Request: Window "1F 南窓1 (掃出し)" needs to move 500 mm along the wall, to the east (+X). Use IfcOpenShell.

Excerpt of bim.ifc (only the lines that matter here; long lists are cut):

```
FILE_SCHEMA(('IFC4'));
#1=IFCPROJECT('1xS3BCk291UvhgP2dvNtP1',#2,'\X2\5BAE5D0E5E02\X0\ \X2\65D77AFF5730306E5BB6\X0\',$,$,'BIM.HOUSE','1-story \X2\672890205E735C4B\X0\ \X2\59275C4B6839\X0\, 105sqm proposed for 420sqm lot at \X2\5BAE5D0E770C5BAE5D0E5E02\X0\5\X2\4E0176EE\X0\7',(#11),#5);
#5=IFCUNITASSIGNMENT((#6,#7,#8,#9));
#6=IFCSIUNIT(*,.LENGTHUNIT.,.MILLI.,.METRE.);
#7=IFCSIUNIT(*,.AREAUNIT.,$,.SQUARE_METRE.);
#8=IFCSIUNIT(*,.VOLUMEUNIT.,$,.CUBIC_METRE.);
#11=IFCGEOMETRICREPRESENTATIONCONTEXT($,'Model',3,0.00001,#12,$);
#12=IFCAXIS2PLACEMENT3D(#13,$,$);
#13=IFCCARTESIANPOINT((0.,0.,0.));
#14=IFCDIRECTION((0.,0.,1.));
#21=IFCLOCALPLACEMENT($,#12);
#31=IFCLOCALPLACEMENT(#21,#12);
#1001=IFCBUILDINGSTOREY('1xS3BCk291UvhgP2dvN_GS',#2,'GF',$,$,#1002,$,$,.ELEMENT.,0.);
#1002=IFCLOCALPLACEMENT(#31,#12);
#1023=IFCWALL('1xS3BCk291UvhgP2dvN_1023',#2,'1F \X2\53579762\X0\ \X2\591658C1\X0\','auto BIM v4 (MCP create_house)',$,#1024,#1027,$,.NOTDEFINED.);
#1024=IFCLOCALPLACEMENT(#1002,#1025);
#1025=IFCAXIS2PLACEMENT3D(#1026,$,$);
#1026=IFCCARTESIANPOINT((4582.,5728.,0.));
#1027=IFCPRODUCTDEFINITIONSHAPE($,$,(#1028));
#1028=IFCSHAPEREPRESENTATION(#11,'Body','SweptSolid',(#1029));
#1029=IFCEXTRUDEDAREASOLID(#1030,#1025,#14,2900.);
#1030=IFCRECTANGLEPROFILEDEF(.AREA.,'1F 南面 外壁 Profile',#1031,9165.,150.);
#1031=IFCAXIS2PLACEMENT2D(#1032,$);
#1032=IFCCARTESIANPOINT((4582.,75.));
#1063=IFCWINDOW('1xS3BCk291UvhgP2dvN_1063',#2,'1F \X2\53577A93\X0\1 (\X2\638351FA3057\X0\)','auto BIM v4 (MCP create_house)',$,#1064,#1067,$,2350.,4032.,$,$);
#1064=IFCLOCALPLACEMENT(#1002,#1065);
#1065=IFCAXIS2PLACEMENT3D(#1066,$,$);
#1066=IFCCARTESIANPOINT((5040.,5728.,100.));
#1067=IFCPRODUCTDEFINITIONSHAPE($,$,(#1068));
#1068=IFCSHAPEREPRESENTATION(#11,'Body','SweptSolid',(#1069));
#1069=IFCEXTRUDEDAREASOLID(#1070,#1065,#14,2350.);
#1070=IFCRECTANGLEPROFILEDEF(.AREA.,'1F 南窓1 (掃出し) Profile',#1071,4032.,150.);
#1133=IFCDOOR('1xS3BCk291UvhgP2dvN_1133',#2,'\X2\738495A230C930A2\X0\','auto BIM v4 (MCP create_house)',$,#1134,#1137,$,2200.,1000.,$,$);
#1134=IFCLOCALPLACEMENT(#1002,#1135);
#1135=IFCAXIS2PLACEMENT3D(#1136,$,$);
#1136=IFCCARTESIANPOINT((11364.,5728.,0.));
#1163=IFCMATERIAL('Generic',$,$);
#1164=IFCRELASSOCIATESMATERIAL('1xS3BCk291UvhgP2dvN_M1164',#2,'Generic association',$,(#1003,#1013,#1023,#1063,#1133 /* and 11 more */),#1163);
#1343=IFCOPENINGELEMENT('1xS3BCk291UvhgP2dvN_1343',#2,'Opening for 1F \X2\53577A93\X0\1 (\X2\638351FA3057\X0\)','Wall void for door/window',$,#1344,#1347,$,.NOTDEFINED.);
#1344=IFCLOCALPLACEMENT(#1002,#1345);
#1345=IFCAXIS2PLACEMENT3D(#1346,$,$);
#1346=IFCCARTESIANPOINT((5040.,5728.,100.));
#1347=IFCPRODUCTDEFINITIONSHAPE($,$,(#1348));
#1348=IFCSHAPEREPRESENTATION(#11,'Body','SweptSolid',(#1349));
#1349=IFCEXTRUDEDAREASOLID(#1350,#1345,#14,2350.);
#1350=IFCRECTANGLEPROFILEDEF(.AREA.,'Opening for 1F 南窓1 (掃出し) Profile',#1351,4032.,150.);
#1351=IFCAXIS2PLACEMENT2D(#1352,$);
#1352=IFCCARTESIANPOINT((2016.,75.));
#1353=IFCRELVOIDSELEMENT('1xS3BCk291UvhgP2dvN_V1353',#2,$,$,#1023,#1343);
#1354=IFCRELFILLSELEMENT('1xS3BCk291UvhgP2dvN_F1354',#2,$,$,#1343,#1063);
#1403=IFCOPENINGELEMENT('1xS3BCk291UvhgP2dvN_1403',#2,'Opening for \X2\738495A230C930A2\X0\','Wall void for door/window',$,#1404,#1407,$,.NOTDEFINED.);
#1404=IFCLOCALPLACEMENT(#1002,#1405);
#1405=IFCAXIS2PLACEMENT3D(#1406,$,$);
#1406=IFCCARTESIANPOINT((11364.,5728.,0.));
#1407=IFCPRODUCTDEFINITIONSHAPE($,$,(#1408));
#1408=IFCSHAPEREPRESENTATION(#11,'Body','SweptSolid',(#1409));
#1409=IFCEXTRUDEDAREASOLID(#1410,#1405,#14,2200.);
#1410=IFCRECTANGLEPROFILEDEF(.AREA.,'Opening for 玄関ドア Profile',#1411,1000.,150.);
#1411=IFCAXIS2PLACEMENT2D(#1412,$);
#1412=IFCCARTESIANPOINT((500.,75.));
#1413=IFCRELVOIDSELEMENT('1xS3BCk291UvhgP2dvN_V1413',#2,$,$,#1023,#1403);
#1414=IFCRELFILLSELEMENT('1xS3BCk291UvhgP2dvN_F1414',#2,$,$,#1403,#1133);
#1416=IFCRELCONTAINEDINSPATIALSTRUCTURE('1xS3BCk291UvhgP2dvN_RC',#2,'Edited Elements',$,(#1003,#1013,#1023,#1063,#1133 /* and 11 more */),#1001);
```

```python
import ifcopenshell
import ifcopenshell.api.geometry
import ifcopenshell.util.placement

model = ifcopenshell.open("bim.ifc")

window = model.by_guid("1xS3BCk291UvhgP2dvN_1063")
opening = window.FillsVoids[0].RelatingOpeningElement
wall = opening.VoidsElements[0].RelatingBuildingElement

wall_matrix = ifcopenshell.util.placement.get_local_placement(wall.ObjectPlacement)
shift = wall_matrix[:3, 0] * 500.0
before = ifcopenshell.util.placement.get_local_placement(window.ObjectPlacement)[:3, 3].copy()

# The window is not placed relative to its opening, so move both.
for product in (opening, window):
    matrix = ifcopenshell.util.placement.get_local_placement(product.ObjectPlacement)
    matrix[:3, 3] += shift
    ifcopenshell.api.geometry.edit_object_placement(model, product=product, matrix=matrix, is_si=False)

after = ifcopenshell.util.placement.get_local_placement(window.ObjectPlacement)[:3, 3]
print("window moved by", (after - before).round(3) + 0.0)

model.write("bim-out.ifc")
```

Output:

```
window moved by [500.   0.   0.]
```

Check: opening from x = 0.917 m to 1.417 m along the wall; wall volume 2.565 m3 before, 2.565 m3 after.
